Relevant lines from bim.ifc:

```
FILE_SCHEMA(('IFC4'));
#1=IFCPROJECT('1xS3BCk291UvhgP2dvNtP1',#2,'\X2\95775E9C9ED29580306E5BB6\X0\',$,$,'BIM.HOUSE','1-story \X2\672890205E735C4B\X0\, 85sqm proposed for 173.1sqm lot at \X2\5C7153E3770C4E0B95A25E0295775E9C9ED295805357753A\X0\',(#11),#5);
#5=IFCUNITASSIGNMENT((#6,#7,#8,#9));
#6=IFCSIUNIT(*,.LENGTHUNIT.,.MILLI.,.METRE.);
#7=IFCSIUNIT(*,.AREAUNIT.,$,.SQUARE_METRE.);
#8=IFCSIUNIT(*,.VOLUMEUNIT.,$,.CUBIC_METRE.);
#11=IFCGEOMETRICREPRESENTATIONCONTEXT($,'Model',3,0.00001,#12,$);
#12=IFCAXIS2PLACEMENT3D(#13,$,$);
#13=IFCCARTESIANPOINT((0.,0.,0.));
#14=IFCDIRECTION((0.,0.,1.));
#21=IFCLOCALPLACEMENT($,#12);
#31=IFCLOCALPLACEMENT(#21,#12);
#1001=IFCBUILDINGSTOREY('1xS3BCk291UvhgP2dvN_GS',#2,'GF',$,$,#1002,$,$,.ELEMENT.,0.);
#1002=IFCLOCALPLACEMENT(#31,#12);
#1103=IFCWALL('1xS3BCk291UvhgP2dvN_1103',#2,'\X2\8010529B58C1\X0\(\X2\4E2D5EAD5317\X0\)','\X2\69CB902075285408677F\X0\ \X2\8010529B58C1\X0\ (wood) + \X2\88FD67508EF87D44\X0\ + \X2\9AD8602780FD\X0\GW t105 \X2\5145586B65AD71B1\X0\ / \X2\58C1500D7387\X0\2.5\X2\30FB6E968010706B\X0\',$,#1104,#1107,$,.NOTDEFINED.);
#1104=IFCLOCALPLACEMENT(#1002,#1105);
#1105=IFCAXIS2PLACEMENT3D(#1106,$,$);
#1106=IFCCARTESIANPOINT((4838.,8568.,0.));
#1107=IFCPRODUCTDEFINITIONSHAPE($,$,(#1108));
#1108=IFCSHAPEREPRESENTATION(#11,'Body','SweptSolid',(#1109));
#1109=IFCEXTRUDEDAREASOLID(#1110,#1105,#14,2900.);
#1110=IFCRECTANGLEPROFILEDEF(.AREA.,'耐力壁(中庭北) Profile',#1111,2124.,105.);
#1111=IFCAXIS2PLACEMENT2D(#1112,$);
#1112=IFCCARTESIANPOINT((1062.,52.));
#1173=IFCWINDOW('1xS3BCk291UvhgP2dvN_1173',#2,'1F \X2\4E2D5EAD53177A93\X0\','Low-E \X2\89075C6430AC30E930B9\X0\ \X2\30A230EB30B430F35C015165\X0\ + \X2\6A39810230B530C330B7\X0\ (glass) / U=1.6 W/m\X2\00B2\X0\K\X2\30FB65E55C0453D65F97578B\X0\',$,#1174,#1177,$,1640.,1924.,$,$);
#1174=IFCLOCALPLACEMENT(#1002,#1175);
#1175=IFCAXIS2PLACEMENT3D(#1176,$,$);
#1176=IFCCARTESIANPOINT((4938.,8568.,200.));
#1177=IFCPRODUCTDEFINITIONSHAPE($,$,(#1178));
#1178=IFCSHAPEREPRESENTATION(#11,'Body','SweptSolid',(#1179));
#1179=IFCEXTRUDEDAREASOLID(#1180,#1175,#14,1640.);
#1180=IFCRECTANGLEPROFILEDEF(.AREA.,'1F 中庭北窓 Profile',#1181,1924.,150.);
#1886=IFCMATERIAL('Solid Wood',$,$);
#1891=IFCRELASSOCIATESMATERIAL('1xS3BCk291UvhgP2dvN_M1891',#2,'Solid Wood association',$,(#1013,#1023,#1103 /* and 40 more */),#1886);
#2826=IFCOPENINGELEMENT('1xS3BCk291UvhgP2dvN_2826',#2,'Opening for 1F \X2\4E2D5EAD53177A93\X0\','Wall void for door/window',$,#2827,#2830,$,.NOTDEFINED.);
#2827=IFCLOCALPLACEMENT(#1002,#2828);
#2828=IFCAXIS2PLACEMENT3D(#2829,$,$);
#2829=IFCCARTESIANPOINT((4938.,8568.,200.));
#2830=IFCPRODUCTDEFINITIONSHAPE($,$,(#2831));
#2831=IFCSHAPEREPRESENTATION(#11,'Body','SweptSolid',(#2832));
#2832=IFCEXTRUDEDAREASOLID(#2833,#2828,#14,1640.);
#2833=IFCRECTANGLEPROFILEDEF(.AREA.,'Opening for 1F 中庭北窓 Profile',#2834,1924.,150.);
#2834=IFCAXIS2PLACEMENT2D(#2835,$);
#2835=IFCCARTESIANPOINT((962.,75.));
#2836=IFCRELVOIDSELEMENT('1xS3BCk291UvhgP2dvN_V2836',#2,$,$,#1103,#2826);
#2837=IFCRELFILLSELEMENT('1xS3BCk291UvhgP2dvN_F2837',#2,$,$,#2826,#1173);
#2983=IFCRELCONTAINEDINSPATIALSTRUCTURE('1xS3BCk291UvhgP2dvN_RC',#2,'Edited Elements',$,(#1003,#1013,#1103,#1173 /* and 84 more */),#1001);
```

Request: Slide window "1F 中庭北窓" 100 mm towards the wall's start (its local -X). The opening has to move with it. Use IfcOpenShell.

```python
import ifcopenshell
import ifcopenshell.api.geometry
import ifcopenshell.util.placement
import ifcopenshell.util.unit

model = ifcopenshell.open("bim.ifc")
unit_scale = ifcopenshell.util.unit.calculate_unit_scale(model)

window = model.by_id(1173)
opening = window.FillsVoids[0].RelatingOpeningElement
wall = opening.VoidsElements[0].RelatingBuildingElement

wall_matrix = ifcopenshell.util.placement.get_local_placement(wall.ObjectPlacement)
shift = wall_matrix[:3, 0] * -0.1 / unit_scale
before = ifcopenshell.util.placement.get_local_placement(window.ObjectPlacement)[:3, 3].copy()

# The window is not placed relative to its opening, so move both.
for product in (opening, window):
    matrix = ifcopenshell.util.placement.get_local_placement(product.ObjectPlacement)
    matrix[:3, 3] += shift
    ifcopenshell.api.geometry.edit_object_placement(model, product=product, matrix=matrix, is_si=False)

after = ifcopenshell.util.placement.get_local_placement(window.ObjectPlacement)[:3, 3]
print("window moved by", (after - before).round(3) + 0.0)

model.write("bim_updated.ifc")
```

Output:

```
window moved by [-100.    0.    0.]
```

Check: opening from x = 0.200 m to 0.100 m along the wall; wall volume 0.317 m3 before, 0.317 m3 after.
